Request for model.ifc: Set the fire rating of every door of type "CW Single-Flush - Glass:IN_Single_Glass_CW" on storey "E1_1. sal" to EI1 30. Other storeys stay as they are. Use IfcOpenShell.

First a look at what the model holds.

```python
import ifcopenshell
import ifcopenshell.util.element

model = ifcopenshell.open("model.ifc")
print(model.schema)
storey = next(s for s in model.by_type("IfcBuildingStorey") if s.Name == "E1_1. sal")
doors = [e for e in ifcopenshell.util.element.get_decomposition(storey) if e.is_a("IfcDoor")]
seen = {}
for e in doors:
    element_type = ifcopenshell.util.element.get_type(e)
    key = (element_type.Name if element_type != e and element_type else None, ifcopenshell.util.element.get_pset(e, "Pset_DoorCommon", "FireRating"))
    seen[key] = seen.get(key, 0) + 1
for (name, value), count in sorted(seen.items(), key=str):
    print(count, "x", name, "|", value)
```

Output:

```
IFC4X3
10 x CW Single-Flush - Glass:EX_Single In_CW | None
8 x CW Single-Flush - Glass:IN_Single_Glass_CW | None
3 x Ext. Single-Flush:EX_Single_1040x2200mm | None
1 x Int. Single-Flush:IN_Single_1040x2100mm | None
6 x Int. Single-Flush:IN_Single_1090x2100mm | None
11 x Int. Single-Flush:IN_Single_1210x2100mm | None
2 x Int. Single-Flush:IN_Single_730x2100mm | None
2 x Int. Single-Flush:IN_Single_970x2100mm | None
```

```python
import ifcopenshell
import ifcopenshell.api.pset
import ifcopenshell.util.element

model = ifcopenshell.open("model.ifc")

storey = next(s for s in model.by_type("IfcBuildingStorey") if s.Name == "E1_1. sal")
doors = [e for e in ifcopenshell.util.element.get_decomposition(storey) if e.is_a("IfcDoor")]

count = 0
for e in doors:
    element_type = ifcopenshell.util.element.get_type(e)
    if element_type in (None, e) or element_type.Name != "CW Single-Flush - Glass:IN_Single_Glass_CW":
        continue
    # add_pset returns the element's existing set when there is one.
    pset = ifcopenshell.api.pset.add_pset(model, product=e, name="Pset_DoorCommon")
    ifcopenshell.api.pset.edit_pset(model, pset=pset, properties={"FireRating": "EI1 30"})
    count += 1

print(count, "doors updated")

model.write("model_updated.ifc")
```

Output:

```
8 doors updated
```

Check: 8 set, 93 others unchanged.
